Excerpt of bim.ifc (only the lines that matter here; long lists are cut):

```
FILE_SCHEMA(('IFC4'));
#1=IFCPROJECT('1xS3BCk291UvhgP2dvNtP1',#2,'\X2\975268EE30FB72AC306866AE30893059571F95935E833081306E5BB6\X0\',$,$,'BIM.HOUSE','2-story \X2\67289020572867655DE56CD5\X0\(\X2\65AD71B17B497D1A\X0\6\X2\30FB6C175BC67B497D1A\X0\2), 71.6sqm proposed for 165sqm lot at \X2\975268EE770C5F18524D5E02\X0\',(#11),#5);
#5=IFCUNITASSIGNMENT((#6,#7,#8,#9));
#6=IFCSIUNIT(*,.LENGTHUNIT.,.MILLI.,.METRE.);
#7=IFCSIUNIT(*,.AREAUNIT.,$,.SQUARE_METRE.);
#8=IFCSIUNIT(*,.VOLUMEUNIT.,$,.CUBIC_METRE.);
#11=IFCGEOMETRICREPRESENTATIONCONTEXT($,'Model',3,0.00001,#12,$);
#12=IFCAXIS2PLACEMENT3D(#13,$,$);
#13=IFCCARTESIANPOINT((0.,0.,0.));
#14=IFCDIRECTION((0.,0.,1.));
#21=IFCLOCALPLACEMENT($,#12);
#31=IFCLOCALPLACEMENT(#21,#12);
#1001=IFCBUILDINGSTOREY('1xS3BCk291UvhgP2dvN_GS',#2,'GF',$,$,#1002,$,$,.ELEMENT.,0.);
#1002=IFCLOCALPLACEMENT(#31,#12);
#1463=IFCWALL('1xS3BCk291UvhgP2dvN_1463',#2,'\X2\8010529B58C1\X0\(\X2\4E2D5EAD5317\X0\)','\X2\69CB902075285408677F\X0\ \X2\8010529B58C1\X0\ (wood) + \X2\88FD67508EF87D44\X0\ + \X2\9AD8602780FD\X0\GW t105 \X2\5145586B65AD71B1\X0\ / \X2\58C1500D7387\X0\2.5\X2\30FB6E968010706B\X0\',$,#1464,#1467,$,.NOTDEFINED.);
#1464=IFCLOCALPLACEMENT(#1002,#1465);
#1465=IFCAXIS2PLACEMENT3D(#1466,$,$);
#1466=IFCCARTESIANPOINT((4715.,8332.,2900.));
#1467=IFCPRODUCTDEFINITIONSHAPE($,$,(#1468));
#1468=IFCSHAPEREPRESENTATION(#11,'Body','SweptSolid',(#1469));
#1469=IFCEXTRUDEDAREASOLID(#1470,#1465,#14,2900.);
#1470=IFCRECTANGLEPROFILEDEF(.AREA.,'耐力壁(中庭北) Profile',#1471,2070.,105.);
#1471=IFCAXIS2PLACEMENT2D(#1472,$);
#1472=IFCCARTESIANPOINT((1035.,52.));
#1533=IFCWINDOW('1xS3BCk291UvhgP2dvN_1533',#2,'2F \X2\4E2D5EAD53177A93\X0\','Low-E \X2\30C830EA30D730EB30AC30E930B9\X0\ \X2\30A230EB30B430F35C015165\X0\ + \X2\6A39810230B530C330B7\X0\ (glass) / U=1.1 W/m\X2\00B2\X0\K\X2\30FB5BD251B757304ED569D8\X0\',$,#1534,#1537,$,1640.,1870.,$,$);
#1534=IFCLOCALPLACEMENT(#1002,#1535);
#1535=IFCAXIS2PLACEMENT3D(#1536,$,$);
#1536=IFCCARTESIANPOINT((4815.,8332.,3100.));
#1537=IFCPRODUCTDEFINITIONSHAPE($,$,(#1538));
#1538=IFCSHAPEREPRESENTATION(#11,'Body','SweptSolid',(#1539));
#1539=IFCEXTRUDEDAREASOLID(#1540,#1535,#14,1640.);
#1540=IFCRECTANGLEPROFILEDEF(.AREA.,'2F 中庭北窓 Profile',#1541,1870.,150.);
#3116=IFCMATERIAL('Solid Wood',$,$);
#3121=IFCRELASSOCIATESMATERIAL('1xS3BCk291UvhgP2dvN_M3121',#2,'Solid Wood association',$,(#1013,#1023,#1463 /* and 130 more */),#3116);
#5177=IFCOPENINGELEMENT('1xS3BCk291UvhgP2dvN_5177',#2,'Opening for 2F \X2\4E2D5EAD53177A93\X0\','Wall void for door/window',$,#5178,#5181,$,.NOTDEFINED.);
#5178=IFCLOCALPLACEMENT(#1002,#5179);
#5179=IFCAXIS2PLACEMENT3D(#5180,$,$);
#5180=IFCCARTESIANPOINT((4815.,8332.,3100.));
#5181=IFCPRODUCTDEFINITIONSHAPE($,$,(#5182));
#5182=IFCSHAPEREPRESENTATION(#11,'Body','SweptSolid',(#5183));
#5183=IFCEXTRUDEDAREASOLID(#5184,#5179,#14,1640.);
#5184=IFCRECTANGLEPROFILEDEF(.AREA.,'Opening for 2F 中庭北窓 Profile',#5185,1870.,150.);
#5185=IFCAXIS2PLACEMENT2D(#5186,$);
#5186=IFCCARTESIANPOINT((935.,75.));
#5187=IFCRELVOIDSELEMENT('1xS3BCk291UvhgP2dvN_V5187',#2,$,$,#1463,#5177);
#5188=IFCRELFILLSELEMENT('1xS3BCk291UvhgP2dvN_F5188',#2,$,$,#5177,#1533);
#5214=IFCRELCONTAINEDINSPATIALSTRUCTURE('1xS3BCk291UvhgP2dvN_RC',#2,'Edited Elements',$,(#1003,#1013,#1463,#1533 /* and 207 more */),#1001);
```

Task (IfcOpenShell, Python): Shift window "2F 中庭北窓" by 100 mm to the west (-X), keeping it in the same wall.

```python
import ifcopenshell
import ifcopenshell.api.geometry
import ifcopenshell.util.placement

model = ifcopenshell.open("bim.ifc")

window = model.by_guid("1xS3BCk291UvhgP2dvN_1533")
opening = window.FillsVoids[0].RelatingOpeningElement
wall = opening.VoidsElements[0].RelatingBuildingElement

wall_matrix = ifcopenshell.util.placement.get_local_placement(wall.ObjectPlacement)
shift = wall_matrix[:3, 0] * -100.0
before = ifcopenshell.util.placement.get_local_placement(window.ObjectPlacement)[:3, 3].copy()

# The window is not placed relative to its opening, so move both.
for product in (opening, window):
    matrix = ifcopenshell.util.placement.get_local_placement(product.ObjectPlacement)
    matrix[:3, 3] += shift
    ifcopenshell.api.geometry.edit_object_placement(model, product=product, matrix=matrix, is_si=False)

after = ifcopenshell.util.placement.get_local_placement(window.ObjectPlacement)[:3, 3]
print("window moved by", (after - before).round(3) + 0.0)

model.write("bim-out.ifc")
```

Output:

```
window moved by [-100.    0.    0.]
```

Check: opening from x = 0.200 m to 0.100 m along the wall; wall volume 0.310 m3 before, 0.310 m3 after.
